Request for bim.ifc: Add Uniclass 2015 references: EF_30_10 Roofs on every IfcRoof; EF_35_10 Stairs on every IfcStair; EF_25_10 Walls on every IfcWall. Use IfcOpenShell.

First a look at what the model holds.

```python
import ifcopenshell

model = ifcopenshell.open("bim.ifc")
print(model.schema)
print("classifications:", [c.Name for c in model.by_type("IfcClassification")])
for ifc_class in ("IfcDoor", "IfcRoof", "IfcStair", "IfcWall", "IfcWindow"):
    print(ifc_class, len(model.by_type(ifc_class)))
```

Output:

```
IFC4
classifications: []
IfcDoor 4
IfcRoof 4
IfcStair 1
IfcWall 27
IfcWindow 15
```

```python
import ifcopenshell
import ifcopenshell.api.classification

model = ifcopenshell.open("bim.ifc")

system = ifcopenshell.api.classification.add_classification(model, classification="Uniclass 2015")

codes = {
    "IfcRoof": ("EF_30_10", "Roofs"),
    "IfcStair": ("EF_35_10", "Stairs"),
    "IfcWall": ("EF_25_10", "Walls"),
}
for ifc_class, (code, name) in codes.items():
    products = model.by_type(ifc_class)
    ifcopenshell.api.classification.add_reference(
        model, products=products, classification=system, identification=code, name=name
    )
    print(code, len(products))

model.write("bim_updated.ifc")
```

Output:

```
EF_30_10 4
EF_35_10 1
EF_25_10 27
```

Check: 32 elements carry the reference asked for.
